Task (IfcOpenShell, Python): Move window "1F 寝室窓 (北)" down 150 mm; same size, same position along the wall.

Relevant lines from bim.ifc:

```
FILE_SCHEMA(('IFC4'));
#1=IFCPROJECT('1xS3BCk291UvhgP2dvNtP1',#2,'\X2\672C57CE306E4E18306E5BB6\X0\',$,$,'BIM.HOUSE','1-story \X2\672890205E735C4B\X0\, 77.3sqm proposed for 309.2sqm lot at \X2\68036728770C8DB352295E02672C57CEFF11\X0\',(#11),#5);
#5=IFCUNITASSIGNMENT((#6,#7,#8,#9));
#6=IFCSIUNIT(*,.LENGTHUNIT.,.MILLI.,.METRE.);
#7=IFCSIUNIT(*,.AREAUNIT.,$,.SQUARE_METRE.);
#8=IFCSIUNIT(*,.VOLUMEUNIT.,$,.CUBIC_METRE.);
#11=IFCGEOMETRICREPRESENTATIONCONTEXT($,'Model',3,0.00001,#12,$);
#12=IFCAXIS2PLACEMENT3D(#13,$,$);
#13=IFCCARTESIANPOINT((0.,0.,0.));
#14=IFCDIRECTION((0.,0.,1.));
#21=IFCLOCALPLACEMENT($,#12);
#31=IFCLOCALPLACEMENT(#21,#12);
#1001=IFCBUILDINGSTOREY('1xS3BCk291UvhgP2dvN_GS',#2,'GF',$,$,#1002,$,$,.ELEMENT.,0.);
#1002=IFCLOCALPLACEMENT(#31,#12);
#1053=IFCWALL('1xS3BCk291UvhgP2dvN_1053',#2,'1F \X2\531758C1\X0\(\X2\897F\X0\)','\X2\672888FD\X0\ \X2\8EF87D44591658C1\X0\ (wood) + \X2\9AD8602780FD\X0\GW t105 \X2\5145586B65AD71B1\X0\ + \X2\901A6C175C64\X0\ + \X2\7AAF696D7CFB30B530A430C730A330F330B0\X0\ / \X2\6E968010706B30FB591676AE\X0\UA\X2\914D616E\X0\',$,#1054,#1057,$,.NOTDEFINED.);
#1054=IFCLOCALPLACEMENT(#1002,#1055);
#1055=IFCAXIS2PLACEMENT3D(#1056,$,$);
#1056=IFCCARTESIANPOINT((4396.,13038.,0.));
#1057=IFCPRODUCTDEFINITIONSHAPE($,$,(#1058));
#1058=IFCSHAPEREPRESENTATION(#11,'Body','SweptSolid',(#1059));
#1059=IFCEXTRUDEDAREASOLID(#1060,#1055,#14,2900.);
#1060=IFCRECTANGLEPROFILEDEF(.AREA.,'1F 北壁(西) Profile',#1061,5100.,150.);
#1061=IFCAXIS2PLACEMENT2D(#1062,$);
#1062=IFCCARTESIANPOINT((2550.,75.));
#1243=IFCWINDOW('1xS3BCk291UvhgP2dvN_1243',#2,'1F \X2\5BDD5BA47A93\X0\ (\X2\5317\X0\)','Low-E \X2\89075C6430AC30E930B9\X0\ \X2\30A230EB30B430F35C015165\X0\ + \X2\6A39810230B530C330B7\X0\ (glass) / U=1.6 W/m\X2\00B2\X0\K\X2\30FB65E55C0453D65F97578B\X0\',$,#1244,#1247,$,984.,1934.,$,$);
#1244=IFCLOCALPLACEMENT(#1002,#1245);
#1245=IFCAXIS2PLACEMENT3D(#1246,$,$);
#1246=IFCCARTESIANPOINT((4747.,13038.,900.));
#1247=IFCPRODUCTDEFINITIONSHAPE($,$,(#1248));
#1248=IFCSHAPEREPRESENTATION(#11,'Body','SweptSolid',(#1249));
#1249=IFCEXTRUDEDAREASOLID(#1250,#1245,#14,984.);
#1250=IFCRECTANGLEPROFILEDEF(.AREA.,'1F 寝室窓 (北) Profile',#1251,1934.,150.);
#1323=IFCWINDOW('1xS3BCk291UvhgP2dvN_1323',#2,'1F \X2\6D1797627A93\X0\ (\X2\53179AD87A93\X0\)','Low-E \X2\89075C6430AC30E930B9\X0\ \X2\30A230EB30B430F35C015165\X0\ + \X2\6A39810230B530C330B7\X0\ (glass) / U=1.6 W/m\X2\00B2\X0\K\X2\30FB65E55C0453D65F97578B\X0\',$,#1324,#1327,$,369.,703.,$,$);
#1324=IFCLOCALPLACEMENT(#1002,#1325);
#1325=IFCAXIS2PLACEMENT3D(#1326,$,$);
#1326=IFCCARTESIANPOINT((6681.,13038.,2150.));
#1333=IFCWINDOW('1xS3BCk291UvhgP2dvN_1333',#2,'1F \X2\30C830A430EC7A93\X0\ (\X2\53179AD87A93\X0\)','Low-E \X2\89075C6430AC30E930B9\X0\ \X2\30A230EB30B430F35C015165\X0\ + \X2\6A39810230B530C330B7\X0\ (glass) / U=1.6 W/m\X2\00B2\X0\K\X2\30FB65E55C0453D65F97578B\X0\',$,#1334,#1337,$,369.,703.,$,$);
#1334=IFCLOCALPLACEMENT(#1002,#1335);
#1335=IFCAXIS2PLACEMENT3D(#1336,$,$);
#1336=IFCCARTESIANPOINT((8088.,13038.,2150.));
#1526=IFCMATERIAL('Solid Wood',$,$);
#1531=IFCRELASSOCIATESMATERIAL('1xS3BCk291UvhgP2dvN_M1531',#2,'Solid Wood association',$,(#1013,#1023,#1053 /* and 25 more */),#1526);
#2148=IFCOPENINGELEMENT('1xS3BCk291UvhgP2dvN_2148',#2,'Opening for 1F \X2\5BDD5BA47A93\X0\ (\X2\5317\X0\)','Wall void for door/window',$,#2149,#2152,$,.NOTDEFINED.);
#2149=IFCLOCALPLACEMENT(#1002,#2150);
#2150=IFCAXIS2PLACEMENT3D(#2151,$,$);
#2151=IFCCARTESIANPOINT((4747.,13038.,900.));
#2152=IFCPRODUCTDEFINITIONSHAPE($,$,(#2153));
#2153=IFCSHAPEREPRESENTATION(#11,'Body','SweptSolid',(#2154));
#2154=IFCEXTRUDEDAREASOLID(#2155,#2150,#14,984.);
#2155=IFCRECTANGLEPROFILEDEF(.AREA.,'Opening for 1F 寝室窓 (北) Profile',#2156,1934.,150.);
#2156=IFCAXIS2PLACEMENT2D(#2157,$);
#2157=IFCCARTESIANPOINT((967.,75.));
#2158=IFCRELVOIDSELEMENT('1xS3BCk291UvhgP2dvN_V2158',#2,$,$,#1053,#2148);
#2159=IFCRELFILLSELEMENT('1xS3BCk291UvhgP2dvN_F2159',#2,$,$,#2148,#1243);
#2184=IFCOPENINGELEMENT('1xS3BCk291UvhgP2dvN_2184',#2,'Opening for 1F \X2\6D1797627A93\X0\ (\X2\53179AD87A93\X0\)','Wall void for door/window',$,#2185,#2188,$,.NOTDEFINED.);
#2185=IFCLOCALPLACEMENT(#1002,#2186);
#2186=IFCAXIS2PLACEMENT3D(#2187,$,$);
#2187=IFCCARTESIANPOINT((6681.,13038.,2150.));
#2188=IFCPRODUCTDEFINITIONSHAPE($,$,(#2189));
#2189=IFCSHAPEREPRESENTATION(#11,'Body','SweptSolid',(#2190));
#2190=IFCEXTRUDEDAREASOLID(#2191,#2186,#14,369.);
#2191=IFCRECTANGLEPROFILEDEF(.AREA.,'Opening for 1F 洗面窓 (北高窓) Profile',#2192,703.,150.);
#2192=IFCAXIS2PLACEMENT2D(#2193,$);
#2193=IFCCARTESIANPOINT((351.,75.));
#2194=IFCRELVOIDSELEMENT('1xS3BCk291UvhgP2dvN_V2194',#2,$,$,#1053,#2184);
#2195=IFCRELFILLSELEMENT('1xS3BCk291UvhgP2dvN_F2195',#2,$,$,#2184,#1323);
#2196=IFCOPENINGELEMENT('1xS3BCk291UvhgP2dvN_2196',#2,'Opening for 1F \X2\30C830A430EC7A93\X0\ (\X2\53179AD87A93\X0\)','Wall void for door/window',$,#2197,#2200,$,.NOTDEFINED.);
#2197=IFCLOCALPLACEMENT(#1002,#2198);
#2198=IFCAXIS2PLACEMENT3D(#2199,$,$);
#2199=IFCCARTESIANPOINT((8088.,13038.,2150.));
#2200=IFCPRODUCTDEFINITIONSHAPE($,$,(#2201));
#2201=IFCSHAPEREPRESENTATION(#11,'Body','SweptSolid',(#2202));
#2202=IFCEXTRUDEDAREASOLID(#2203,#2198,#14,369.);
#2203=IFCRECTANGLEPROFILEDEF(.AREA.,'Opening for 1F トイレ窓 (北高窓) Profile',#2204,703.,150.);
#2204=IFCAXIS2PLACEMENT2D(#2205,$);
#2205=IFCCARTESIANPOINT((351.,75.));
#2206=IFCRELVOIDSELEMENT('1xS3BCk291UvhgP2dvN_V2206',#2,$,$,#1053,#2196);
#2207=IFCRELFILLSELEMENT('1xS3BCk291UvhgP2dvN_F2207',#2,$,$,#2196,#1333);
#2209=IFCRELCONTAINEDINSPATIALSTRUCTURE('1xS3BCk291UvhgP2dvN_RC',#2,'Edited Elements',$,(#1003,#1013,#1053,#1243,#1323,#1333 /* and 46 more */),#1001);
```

```python
import numpy as np
import ifcopenshell
import ifcopenshell.api.geometry
import ifcopenshell.util.placement
import ifcopenshell.util.unit

model = ifcopenshell.open("bim.ifc")
unit_scale = ifcopenshell.util.unit.calculate_unit_scale(model)

window = model.by_id(1243)
opening = window.FillsVoids[0].RelatingOpeningElement
dz = -0.15 / unit_scale

shift = np.array([0.0, 0.0, dz])
# The window is not placed relative to its opening, so move both.
for product in (opening, window):
    matrix = ifcopenshell.util.placement.get_local_placement(product.ObjectPlacement)
    matrix[:3, 3] += shift
    ifcopenshell.api.geometry.edit_object_placement(model, product=product, matrix=matrix, is_si=False)

print(f"moved by {dz * unit_scale:+.3f} m")

model.write("bim_v2.ifc")
```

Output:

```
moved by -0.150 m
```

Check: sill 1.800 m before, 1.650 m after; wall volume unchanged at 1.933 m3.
